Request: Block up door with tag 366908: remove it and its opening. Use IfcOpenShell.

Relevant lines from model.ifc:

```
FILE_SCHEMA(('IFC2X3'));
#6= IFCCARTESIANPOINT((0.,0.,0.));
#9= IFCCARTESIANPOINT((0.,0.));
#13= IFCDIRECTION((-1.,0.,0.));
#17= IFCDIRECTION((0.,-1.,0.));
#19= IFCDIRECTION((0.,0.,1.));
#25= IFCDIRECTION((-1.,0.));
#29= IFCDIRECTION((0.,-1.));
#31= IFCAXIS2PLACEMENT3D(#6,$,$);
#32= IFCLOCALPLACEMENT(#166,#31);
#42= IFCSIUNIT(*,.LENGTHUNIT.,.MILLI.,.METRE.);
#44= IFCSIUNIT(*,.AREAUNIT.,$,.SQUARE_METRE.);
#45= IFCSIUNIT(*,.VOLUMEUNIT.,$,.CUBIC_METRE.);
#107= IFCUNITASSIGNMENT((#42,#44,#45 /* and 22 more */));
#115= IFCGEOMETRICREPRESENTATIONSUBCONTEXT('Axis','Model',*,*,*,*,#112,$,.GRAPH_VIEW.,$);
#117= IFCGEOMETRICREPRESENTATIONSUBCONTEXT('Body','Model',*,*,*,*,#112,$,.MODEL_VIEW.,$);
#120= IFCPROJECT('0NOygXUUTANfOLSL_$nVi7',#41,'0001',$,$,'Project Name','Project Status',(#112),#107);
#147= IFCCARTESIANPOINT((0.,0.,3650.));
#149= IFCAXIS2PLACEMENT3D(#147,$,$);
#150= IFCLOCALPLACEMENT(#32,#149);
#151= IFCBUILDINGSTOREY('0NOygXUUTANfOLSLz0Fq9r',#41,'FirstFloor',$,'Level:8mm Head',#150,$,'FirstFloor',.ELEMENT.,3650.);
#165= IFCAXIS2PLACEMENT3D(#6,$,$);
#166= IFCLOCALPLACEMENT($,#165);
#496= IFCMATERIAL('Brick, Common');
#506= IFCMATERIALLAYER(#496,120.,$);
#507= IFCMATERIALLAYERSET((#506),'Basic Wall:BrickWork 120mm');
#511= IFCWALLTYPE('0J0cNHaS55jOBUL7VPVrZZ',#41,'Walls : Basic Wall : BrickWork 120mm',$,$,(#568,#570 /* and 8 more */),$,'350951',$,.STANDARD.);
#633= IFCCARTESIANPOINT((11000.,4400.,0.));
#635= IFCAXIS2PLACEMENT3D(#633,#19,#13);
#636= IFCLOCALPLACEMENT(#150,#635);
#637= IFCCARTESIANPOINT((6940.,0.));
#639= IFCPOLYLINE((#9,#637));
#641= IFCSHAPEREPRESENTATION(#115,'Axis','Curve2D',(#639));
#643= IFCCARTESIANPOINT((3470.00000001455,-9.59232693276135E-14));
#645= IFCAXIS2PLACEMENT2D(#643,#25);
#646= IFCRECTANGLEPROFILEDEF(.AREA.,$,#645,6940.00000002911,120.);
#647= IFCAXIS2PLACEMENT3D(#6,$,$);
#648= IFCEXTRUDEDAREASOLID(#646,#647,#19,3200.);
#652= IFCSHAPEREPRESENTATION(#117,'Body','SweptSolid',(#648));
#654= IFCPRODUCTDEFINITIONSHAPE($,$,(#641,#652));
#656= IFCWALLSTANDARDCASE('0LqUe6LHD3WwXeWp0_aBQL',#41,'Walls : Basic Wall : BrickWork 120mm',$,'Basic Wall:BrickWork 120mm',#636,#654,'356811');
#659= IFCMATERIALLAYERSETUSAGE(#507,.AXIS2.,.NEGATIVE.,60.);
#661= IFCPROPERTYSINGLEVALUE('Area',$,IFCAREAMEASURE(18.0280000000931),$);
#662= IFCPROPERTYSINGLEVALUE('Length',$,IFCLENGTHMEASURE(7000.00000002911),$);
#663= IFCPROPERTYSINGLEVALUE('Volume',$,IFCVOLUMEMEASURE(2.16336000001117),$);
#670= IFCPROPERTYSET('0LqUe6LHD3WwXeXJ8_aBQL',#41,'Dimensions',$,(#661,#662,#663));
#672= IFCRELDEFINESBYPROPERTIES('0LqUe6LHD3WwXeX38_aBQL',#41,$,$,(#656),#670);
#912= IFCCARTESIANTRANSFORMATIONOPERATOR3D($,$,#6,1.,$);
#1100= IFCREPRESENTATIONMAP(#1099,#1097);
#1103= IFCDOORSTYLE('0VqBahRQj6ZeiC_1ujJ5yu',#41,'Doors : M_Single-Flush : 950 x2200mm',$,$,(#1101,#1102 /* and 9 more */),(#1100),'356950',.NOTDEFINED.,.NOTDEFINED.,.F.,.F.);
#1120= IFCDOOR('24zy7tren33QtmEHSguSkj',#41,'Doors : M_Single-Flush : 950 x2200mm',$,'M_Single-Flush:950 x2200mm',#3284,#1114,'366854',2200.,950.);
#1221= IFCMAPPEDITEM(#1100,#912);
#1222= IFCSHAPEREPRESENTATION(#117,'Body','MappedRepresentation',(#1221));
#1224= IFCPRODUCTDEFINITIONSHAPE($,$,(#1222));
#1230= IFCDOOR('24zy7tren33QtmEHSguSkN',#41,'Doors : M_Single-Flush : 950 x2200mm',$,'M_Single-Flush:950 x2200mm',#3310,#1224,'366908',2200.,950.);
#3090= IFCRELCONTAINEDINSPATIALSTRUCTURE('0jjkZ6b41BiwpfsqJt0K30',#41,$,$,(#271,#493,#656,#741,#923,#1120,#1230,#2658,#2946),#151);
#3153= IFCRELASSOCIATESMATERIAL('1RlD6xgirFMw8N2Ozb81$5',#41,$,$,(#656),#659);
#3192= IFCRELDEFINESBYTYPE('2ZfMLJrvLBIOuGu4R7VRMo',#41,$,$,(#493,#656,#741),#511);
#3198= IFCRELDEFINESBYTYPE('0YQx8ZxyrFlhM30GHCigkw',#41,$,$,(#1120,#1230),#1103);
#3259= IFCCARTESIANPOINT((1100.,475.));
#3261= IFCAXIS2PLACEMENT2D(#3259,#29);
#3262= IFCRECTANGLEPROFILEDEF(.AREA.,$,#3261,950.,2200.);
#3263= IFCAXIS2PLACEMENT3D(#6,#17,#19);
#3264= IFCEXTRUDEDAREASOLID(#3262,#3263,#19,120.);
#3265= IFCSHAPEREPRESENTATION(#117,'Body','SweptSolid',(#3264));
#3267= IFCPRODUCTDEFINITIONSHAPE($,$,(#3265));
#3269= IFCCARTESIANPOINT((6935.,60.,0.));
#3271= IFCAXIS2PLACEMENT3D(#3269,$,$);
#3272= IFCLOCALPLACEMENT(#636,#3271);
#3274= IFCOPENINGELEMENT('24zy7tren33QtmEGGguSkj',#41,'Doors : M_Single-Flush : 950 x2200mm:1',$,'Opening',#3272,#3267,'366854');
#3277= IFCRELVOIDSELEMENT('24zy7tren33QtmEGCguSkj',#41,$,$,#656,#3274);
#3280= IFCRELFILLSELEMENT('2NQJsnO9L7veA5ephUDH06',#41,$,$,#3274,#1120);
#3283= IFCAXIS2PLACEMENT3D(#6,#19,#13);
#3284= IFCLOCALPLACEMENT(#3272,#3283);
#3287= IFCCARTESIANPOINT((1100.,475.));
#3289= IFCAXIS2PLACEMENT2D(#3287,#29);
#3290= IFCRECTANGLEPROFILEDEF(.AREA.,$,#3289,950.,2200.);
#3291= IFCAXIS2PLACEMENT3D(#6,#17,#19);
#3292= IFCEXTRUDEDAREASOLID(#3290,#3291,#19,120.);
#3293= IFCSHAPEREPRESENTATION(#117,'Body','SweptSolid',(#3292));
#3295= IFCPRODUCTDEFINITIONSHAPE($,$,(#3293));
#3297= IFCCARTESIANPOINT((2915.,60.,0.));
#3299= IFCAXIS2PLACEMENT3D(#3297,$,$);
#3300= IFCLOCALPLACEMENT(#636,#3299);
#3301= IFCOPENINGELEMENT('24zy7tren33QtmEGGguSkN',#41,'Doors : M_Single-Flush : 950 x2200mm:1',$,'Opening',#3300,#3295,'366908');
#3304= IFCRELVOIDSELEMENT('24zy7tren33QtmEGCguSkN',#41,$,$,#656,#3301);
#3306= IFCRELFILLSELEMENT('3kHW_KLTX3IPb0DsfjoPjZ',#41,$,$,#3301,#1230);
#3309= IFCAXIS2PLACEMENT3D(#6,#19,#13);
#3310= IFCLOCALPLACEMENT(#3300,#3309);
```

```python
import ifcopenshell
import ifcopenshell.api.feature
import ifcopenshell.api.pset
import ifcopenshell.api.root
import ifcopenshell.geom
import ifcopenshell.util.element
import ifcopenshell.util.shape
import ifcopenshell.util.unit

model = ifcopenshell.open("model.ifc")
area_scale = ifcopenshell.util.unit.calculate_unit_scale(model, "AREAUNIT")
volume_scale = ifcopenshell.util.unit.calculate_unit_scale(model, "VOLUMEUNIT")
settings = ifcopenshell.geom.settings()


def volume(element):
    """Net volume in cubic metres, openings subtracted."""
    shape = ifcopenshell.geom.create_shape(settings, element)
    return ifcopenshell.util.shape.get_volume(shape.geometry)


door = model.by_id(1230)
opening = door.FillsVoids[0].RelatingOpeningElement
wall = opening.VoidsElements[0].RelatingBuildingElement
before = volume(wall)

ifcopenshell.api.root.remove_product(model, product=door)
ifcopenshell.api.feature.remove_feature(model, feature=opening)

after = volume(wall)
thickness = 0.12  # wall thickness in metres

# Update the wall's stored quantities.
pset = model.by_id(ifcopenshell.util.element.get_pset(wall, "Dimensions", should_inherit=False)["id"])
ifcopenshell.api.pset.edit_pset(model, pset=pset, properties={
    "Area": model.create_entity("IfcAreaMeasure", after / thickness / area_scale),
    "Volume": model.create_entity("IfcVolumeMeasure", after / volume_scale),
})

print(f"wall volume {before:.3f} -> {after:.3f} m3")

model.write("model_updated.ifc")
```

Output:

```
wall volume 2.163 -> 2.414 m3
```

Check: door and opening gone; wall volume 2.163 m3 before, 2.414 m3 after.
